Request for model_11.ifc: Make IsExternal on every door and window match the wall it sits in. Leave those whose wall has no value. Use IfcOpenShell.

First a look at what the model holds.

```python
import ifcopenshell
import ifcopenshell.util.element

model = ifcopenshell.open("model_11.ifc")
print(model.schema)
seen = {}
for e in model.by_type("IfcDoor") + model.by_type("IfcWindow"):
    if not e.FillsVoids:
        continue
    host = e.FillsVoids[0].RelatingOpeningElement.VoidsElements[0].RelatingBuildingElement
    own = ifcopenshell.util.element.get_pset(e, f"Pset_{e.is_a()[3:].removesuffix('StandardCase')}Common", "IsExternal")
    wall = ifcopenshell.util.element.get_pset(host, "Pset_WallCommon", "IsExternal")
    seen[e.is_a(), own, wall] = seen.get((e.is_a(), own, wall), 0) + 1
for (cls, own, wall), count in sorted(seen.items(), key=str):
    print(count, cls, "IsExternal:", own, "| host wall:", wall)
```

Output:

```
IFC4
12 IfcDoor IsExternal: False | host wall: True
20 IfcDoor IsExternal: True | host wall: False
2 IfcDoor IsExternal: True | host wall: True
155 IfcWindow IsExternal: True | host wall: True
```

```python
import ifcopenshell
import ifcopenshell.api.pset
import ifcopenshell.util.element

model = ifcopenshell.open("model_11.ifc")

count = 0
for ifc_class, pset_name in (("IfcDoor", "Pset_DoorCommon"), ("IfcWindow", "Pset_WindowCommon")):
    for e in model.by_type(ifc_class):
        if not e.FillsVoids:
            continue
        host = e.FillsVoids[0].RelatingOpeningElement.VoidsElements[0].RelatingBuildingElement
        external = ifcopenshell.util.element.get_pset(host, "Pset_WallCommon", "IsExternal")
        if external is None or ifcopenshell.util.element.get_pset(e, pset_name, "IsExternal") == external:
            continue
        pset = ifcopenshell.api.pset.add_pset(model, product=e, name=pset_name)
        ifcopenshell.api.pset.edit_pset(model, pset=pset, properties={"IsExternal": external})
        count += 1

print(count, "updated")

model.write("model_11_edited.ifc")
```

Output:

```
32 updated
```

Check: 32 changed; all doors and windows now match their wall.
